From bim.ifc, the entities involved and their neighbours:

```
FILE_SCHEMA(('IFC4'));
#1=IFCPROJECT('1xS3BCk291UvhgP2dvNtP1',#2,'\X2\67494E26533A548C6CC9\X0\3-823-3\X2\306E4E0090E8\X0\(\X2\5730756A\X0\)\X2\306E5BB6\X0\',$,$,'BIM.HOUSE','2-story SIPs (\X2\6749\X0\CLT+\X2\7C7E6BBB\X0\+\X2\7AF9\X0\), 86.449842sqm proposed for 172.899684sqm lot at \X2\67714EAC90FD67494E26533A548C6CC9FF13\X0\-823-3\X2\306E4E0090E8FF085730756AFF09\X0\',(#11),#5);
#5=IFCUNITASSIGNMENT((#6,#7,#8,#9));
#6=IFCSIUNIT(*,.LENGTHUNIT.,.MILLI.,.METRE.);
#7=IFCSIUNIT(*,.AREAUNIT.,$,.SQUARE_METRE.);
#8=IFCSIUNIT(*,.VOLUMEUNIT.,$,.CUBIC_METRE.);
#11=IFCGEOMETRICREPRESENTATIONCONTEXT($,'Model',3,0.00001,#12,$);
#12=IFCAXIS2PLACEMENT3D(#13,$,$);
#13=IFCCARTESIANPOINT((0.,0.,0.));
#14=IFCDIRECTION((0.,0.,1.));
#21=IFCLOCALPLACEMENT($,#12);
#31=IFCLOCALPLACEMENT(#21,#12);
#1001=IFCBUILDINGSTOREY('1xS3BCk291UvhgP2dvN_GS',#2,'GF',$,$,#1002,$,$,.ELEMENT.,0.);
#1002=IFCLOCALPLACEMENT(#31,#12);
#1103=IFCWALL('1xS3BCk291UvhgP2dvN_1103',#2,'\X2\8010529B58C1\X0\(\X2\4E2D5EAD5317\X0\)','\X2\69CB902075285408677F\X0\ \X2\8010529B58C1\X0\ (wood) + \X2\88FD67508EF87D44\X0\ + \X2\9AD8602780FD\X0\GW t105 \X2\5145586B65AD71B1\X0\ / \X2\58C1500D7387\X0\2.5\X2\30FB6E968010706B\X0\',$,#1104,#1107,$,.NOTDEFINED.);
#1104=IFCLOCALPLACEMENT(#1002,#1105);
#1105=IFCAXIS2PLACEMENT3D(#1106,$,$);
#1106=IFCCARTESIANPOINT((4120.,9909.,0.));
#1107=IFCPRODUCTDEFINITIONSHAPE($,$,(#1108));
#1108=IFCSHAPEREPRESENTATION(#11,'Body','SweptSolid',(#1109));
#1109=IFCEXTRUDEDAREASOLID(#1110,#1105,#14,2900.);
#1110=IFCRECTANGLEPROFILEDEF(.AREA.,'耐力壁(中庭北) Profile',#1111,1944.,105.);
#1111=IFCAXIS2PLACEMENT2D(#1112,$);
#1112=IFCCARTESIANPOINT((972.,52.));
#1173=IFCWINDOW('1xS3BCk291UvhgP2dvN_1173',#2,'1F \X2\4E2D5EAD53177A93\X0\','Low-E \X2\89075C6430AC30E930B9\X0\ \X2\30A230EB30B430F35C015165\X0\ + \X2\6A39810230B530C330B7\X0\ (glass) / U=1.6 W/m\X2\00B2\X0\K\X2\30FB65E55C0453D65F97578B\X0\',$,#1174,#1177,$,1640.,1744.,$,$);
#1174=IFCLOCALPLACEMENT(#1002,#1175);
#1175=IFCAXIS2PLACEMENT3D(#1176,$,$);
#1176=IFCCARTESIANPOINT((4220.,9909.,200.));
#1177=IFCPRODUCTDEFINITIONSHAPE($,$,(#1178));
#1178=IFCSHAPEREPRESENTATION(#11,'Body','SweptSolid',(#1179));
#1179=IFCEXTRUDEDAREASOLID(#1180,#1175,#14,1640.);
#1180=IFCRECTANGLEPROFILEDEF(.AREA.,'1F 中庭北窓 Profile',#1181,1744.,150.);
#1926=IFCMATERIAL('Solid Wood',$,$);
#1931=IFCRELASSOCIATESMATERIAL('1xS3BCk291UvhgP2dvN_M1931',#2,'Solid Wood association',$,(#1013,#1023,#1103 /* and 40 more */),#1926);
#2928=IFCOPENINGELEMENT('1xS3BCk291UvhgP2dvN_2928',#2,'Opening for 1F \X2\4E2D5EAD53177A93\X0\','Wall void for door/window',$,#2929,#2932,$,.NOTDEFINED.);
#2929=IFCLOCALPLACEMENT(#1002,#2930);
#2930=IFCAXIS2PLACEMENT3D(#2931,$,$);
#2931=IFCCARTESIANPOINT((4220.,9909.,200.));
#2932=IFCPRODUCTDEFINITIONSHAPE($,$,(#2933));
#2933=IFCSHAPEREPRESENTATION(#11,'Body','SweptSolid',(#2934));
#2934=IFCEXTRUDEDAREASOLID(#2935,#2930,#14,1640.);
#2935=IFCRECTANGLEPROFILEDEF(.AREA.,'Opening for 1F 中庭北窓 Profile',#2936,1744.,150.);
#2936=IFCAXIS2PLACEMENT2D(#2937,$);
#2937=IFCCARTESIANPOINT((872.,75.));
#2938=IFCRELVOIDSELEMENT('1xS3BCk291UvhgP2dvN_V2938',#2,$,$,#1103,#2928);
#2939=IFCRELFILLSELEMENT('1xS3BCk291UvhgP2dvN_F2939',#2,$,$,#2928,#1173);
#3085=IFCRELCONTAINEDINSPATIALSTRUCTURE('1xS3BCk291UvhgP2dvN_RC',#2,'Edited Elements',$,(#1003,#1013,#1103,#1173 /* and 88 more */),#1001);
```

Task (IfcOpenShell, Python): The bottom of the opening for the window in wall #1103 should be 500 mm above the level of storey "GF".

```python
import numpy as np
import ifcopenshell
import ifcopenshell.api.geometry
import ifcopenshell.geom
import ifcopenshell.util.element
import ifcopenshell.util.placement
import ifcopenshell.util.shape
import ifcopenshell.util.unit

model = ifcopenshell.open("bim.ifc")
unit_scale = ifcopenshell.util.unit.calculate_unit_scale(model)

window = model.by_id(1173)
opening = window.FillsVoids[0].RelatingOpeningElement
storey = ifcopenshell.util.element.get_container(window, ifc_class="IfcBuildingStorey")
level = ifcopenshell.util.placement.get_local_placement(storey.ObjectPlacement)[2, 3]

# The opening's origin need not be at the sill, so measure its lowest point.
shape = ifcopenshell.geom.create_shape(ifcopenshell.geom.settings(), opening)
bottom = ifcopenshell.util.shape.get_shape_bottom_elevation(shape, shape.geometry) / unit_scale
dz = level + 0.5 / unit_scale - bottom

shift = np.array([0.0, 0.0, dz])
# The window is not placed relative to its opening, so move both.
for product in (opening, window):
    matrix = ifcopenshell.util.placement.get_local_placement(product.ObjectPlacement)
    matrix[:3, 3] += shift
    ifcopenshell.api.geometry.edit_object_placement(model, product=product, matrix=matrix, is_si=False)

print(f"moved by {dz * unit_scale:+.3f} m")

model.write("bim_edited.ifc")
```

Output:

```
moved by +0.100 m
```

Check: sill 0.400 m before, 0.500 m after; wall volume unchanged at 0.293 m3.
